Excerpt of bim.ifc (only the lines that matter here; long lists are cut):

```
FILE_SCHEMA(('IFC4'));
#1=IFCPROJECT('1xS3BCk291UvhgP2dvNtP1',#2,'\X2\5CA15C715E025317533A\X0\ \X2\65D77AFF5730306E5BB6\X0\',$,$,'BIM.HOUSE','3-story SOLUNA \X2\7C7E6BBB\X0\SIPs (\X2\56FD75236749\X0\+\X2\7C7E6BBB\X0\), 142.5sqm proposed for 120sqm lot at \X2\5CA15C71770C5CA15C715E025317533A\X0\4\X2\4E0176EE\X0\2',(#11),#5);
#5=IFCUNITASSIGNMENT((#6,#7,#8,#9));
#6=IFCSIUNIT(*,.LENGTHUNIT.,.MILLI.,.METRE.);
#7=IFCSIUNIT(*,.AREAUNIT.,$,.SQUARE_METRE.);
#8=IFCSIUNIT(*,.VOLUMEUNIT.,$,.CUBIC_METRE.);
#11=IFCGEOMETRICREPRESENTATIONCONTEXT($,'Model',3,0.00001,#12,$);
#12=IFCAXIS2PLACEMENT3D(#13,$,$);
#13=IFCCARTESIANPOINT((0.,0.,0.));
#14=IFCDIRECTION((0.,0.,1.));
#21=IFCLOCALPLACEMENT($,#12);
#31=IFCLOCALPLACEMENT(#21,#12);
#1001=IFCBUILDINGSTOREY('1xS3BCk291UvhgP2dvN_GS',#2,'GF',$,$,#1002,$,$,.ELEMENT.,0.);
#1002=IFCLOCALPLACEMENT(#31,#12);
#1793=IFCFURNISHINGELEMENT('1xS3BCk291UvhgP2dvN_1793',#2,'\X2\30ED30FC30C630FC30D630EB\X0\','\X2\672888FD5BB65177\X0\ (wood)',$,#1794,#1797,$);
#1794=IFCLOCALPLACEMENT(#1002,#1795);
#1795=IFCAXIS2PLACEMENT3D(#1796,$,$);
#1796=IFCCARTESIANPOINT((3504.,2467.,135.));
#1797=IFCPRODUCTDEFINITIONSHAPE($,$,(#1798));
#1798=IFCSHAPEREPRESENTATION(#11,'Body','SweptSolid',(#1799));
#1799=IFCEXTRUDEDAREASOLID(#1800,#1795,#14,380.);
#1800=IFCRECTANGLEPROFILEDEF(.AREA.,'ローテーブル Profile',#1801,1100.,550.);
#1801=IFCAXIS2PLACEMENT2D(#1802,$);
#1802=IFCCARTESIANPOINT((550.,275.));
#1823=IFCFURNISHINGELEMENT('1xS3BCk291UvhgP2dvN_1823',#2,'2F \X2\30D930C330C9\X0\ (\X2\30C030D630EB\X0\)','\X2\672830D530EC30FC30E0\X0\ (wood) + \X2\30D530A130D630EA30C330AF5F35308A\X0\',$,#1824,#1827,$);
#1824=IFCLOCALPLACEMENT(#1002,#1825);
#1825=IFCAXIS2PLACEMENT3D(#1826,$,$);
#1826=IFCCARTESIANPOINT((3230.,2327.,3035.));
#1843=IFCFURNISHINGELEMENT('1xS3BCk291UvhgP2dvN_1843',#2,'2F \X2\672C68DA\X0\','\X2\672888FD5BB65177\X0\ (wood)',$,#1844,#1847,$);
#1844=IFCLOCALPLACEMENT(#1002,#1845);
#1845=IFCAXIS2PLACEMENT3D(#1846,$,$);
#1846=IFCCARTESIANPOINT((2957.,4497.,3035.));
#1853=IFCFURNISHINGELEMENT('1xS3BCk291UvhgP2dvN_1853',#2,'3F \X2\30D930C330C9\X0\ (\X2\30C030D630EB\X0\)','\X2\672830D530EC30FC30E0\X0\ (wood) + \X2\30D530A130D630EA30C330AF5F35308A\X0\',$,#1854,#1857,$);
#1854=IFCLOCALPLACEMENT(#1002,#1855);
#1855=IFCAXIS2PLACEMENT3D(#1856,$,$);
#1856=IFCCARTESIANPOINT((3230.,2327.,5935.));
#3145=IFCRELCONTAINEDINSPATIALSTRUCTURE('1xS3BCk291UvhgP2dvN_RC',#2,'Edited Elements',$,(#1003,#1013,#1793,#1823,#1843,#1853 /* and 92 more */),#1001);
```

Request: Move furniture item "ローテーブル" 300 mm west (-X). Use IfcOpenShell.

```python
import ifcopenshell
import ifcopenshell.api.geometry
import ifcopenshell.util.placement

model = ifcopenshell.open("bim.ifc")

item = model.by_guid("1xS3BCk291UvhgP2dvN_1793")
matrix = ifcopenshell.util.placement.get_local_placement(item.ObjectPlacement)
matrix[0, 3] -= 300.0
ifcopenshell.api.geometry.edit_object_placement(model, product=item, matrix=matrix, is_si=False)

print(ifcopenshell.util.placement.get_local_placement(item.ObjectPlacement).round(3) + 0.0)

model.write("bim_updated.ifc")
```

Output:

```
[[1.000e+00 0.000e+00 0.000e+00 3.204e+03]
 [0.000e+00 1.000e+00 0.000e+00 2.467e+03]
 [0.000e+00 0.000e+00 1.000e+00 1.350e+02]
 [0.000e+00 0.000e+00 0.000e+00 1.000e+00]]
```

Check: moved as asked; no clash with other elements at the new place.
